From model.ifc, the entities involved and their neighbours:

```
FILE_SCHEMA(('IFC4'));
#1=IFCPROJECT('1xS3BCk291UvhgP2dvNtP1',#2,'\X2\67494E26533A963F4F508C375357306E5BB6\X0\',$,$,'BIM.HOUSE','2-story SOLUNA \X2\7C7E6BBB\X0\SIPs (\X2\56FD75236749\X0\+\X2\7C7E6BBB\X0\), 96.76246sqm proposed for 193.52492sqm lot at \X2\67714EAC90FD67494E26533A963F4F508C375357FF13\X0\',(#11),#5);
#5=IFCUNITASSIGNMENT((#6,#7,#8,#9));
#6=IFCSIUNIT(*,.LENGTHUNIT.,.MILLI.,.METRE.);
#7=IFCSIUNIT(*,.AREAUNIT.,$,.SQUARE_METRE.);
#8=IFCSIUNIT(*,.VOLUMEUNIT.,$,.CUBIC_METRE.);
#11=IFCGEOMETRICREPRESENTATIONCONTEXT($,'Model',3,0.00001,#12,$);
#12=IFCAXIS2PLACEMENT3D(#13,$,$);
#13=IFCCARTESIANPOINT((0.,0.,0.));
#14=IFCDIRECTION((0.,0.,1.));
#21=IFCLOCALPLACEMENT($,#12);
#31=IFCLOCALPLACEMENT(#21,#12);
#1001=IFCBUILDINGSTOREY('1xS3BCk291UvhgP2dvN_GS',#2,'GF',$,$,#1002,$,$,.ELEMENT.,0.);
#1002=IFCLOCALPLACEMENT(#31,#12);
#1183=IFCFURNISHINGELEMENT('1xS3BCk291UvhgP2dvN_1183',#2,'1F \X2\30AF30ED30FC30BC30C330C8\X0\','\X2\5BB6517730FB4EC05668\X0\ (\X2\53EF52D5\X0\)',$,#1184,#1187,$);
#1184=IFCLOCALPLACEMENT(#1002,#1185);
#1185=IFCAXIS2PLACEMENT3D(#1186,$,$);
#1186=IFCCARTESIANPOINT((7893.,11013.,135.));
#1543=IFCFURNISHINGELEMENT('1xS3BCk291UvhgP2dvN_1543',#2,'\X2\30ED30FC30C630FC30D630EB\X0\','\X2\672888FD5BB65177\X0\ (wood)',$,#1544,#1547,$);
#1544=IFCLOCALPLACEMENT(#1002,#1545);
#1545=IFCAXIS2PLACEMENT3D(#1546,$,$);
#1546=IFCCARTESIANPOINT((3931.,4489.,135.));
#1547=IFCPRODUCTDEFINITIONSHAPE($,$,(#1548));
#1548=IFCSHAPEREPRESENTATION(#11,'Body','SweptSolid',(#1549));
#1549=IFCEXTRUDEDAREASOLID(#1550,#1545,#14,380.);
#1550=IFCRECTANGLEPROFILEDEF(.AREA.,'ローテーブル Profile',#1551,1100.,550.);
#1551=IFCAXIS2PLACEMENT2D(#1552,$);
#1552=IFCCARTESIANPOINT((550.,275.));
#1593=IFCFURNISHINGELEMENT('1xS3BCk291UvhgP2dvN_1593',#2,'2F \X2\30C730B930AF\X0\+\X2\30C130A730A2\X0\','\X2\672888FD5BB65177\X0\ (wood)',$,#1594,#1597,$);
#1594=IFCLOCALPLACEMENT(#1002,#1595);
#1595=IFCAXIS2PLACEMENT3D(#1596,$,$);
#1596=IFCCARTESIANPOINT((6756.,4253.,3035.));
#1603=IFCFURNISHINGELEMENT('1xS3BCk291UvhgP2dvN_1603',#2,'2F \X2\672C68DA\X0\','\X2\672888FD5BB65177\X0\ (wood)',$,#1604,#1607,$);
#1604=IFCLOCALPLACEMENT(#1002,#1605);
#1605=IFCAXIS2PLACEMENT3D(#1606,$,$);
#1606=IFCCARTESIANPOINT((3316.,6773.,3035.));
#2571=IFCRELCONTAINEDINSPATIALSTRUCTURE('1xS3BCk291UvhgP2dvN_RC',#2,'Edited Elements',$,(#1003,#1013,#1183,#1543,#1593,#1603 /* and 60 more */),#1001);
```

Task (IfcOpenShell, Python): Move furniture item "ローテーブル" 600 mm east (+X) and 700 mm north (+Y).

```python
import ifcopenshell
import ifcopenshell.api.geometry
import ifcopenshell.util.placement
import ifcopenshell.util.unit

model = ifcopenshell.open("model.ifc")
unit_scale = ifcopenshell.util.unit.calculate_unit_scale(model)

item = model.by_guid("1xS3BCk291UvhgP2dvN_1543")
matrix = ifcopenshell.util.placement.get_local_placement(item.ObjectPlacement)
matrix[0, 3] += 0.6 / unit_scale
matrix[1, 3] += 0.7 / unit_scale
ifcopenshell.api.geometry.edit_object_placement(model, product=item, matrix=matrix, is_si=False)

print(ifcopenshell.util.placement.get_local_placement(item.ObjectPlacement).round(3) + 0.0)

model.write("model_v2.ifc")
```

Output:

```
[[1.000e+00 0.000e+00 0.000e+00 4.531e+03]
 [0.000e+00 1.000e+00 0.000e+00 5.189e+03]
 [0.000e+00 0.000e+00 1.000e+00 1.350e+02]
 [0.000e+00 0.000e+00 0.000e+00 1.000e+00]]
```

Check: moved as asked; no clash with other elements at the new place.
